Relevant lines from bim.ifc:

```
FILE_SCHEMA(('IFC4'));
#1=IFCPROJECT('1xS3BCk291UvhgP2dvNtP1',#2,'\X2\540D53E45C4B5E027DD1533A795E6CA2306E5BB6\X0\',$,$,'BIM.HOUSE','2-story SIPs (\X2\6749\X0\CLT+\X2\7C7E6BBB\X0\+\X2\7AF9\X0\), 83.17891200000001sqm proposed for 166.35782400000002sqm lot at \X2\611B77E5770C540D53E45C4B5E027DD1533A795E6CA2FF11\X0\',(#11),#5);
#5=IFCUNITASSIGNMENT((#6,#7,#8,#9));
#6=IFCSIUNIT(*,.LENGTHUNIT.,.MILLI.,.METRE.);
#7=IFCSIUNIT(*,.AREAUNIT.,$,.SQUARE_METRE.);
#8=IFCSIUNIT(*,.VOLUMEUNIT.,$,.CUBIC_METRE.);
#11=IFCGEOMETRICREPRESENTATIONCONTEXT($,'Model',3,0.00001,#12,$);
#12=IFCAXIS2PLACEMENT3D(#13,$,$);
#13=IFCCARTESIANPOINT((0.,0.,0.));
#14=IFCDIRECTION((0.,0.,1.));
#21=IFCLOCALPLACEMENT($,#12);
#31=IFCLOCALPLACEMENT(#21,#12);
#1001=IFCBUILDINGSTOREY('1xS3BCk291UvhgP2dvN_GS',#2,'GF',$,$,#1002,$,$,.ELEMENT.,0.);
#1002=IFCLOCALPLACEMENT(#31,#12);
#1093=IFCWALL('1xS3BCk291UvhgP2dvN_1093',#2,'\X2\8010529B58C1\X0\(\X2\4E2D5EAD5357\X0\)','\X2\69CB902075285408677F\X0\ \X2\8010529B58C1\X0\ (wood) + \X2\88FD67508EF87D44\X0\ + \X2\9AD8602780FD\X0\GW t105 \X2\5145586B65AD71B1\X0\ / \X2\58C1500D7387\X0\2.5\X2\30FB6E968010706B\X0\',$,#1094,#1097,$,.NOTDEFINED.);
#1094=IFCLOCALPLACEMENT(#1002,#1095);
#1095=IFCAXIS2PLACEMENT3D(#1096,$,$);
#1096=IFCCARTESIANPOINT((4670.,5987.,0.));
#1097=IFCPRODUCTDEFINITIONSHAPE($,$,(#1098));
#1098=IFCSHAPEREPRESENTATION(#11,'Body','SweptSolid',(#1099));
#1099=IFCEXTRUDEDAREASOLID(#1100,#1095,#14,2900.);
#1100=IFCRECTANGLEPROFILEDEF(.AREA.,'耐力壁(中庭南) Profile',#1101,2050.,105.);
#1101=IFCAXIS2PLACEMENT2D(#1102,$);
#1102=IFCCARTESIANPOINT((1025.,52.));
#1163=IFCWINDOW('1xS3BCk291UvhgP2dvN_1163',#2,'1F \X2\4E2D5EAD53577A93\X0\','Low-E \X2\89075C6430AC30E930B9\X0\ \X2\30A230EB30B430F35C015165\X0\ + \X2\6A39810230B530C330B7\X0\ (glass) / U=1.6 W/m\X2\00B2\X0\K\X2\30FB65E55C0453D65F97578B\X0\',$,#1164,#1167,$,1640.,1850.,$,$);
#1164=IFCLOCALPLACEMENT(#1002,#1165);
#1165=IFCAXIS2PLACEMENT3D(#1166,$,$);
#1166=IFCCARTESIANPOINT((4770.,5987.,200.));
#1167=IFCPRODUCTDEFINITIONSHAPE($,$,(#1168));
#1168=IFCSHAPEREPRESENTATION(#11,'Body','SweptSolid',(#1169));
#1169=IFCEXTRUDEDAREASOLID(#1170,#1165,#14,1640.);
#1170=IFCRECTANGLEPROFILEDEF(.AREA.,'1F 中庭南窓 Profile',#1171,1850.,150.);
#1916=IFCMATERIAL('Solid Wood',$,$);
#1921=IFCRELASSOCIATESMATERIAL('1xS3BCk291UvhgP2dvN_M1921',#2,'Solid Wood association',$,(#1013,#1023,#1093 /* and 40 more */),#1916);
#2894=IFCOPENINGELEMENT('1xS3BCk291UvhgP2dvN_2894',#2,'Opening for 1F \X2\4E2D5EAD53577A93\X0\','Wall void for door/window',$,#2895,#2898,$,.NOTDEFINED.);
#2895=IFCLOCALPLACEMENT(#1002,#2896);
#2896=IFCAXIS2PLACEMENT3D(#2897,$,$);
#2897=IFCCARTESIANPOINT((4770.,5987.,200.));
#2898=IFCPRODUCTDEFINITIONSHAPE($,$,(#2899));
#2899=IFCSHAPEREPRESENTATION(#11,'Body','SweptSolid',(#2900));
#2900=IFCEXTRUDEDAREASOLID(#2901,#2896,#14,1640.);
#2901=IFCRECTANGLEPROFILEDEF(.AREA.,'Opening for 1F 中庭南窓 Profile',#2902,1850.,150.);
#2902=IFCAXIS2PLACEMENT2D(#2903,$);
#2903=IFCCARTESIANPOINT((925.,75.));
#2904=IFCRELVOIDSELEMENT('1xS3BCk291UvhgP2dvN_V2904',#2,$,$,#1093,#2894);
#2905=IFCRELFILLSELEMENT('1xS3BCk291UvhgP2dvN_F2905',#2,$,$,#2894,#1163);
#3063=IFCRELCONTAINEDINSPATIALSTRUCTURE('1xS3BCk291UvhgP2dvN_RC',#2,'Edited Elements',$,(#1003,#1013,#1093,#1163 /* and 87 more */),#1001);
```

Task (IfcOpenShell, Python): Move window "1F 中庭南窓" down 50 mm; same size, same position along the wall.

```python
import numpy as np
import ifcopenshell
import ifcopenshell.api.geometry
import ifcopenshell.util.placement
import ifcopenshell.util.unit

model = ifcopenshell.open("bim.ifc")
unit_scale = ifcopenshell.util.unit.calculate_unit_scale(model)

window = model.by_id(1163)
opening = window.FillsVoids[0].RelatingOpeningElement
dz = -50.0

shift = np.array([0.0, 0.0, dz])
# The window is not placed relative to its opening, so move both.
for product in (opening, window):
    matrix = ifcopenshell.util.placement.get_local_placement(product.ObjectPlacement)
    matrix[:3, 3] += shift
    ifcopenshell.api.geometry.edit_object_placement(model, product=product, matrix=matrix, is_si=False)

print(f"moved by {dz * unit_scale:+.3f} m")

model.write("bim_rev.ifc")
```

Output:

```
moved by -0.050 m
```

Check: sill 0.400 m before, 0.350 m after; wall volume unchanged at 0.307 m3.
